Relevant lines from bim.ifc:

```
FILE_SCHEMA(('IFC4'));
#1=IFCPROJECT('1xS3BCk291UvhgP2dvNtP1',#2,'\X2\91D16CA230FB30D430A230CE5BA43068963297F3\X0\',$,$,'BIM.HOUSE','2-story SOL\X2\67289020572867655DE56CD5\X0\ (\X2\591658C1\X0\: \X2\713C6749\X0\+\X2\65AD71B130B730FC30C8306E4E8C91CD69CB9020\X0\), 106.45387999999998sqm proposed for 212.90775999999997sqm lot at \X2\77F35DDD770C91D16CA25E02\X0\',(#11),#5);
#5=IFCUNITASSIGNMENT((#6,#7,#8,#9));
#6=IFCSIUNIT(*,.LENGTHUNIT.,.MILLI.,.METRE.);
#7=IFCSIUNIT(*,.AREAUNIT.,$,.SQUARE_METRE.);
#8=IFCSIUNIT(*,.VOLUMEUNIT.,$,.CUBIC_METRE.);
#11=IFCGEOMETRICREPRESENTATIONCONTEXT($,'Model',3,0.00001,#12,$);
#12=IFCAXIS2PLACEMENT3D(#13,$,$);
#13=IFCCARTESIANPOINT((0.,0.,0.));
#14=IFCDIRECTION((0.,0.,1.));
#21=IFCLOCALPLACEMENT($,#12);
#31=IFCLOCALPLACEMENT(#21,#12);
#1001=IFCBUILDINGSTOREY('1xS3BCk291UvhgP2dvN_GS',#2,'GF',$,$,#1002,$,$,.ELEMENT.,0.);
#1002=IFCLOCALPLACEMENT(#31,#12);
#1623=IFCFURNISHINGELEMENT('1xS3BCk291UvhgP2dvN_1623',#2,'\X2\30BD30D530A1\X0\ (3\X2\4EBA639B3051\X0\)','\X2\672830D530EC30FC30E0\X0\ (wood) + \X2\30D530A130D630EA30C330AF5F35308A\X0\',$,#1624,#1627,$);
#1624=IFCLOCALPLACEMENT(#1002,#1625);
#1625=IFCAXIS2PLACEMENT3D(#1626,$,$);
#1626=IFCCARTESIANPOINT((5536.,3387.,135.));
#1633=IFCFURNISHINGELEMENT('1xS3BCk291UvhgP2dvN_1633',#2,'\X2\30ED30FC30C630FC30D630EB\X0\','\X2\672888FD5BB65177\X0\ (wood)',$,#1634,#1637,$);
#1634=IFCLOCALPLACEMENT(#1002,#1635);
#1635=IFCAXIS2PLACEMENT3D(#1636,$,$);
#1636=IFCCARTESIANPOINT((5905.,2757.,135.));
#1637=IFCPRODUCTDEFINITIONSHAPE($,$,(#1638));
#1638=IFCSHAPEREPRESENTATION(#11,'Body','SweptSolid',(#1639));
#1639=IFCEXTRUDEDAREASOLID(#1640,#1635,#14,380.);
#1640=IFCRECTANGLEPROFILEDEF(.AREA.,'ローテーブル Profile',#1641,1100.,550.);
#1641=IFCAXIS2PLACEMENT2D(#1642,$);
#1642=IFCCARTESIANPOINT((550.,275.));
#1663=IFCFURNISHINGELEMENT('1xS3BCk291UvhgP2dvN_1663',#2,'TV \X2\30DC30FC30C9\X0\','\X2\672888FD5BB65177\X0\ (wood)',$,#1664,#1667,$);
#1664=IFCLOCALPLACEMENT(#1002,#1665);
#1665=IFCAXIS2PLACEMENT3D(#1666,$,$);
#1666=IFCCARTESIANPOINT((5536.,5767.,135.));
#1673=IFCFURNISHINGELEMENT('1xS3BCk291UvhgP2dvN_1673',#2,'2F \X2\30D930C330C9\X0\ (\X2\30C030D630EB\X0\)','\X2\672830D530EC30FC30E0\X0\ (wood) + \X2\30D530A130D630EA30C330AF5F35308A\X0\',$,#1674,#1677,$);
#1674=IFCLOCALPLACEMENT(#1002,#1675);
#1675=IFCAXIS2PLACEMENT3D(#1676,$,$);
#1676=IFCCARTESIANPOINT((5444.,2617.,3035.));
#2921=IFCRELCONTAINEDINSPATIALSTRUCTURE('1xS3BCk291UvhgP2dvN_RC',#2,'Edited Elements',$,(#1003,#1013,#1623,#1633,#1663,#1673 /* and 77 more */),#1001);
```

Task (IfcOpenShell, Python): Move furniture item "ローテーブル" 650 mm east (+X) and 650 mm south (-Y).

```python
import ifcopenshell
import ifcopenshell.api.geometry
import ifcopenshell.util.placement
import ifcopenshell.util.unit

model = ifcopenshell.open("bim.ifc")
unit_scale = ifcopenshell.util.unit.calculate_unit_scale(model)

item = model.by_guid("1xS3BCk291UvhgP2dvN_1633")
matrix = ifcopenshell.util.placement.get_local_placement(item.ObjectPlacement)
matrix[0, 3] += 0.65 / unit_scale
matrix[1, 3] -= 0.65 / unit_scale
ifcopenshell.api.geometry.edit_object_placement(model, product=item, matrix=matrix, is_si=False)

print(ifcopenshell.util.placement.get_local_placement(item.ObjectPlacement).round(3) + 0.0)

model.write("bim_edited.ifc")
```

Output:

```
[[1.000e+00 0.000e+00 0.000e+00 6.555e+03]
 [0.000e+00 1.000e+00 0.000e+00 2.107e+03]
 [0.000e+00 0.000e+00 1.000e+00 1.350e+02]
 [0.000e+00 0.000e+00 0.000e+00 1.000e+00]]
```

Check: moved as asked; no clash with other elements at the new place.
